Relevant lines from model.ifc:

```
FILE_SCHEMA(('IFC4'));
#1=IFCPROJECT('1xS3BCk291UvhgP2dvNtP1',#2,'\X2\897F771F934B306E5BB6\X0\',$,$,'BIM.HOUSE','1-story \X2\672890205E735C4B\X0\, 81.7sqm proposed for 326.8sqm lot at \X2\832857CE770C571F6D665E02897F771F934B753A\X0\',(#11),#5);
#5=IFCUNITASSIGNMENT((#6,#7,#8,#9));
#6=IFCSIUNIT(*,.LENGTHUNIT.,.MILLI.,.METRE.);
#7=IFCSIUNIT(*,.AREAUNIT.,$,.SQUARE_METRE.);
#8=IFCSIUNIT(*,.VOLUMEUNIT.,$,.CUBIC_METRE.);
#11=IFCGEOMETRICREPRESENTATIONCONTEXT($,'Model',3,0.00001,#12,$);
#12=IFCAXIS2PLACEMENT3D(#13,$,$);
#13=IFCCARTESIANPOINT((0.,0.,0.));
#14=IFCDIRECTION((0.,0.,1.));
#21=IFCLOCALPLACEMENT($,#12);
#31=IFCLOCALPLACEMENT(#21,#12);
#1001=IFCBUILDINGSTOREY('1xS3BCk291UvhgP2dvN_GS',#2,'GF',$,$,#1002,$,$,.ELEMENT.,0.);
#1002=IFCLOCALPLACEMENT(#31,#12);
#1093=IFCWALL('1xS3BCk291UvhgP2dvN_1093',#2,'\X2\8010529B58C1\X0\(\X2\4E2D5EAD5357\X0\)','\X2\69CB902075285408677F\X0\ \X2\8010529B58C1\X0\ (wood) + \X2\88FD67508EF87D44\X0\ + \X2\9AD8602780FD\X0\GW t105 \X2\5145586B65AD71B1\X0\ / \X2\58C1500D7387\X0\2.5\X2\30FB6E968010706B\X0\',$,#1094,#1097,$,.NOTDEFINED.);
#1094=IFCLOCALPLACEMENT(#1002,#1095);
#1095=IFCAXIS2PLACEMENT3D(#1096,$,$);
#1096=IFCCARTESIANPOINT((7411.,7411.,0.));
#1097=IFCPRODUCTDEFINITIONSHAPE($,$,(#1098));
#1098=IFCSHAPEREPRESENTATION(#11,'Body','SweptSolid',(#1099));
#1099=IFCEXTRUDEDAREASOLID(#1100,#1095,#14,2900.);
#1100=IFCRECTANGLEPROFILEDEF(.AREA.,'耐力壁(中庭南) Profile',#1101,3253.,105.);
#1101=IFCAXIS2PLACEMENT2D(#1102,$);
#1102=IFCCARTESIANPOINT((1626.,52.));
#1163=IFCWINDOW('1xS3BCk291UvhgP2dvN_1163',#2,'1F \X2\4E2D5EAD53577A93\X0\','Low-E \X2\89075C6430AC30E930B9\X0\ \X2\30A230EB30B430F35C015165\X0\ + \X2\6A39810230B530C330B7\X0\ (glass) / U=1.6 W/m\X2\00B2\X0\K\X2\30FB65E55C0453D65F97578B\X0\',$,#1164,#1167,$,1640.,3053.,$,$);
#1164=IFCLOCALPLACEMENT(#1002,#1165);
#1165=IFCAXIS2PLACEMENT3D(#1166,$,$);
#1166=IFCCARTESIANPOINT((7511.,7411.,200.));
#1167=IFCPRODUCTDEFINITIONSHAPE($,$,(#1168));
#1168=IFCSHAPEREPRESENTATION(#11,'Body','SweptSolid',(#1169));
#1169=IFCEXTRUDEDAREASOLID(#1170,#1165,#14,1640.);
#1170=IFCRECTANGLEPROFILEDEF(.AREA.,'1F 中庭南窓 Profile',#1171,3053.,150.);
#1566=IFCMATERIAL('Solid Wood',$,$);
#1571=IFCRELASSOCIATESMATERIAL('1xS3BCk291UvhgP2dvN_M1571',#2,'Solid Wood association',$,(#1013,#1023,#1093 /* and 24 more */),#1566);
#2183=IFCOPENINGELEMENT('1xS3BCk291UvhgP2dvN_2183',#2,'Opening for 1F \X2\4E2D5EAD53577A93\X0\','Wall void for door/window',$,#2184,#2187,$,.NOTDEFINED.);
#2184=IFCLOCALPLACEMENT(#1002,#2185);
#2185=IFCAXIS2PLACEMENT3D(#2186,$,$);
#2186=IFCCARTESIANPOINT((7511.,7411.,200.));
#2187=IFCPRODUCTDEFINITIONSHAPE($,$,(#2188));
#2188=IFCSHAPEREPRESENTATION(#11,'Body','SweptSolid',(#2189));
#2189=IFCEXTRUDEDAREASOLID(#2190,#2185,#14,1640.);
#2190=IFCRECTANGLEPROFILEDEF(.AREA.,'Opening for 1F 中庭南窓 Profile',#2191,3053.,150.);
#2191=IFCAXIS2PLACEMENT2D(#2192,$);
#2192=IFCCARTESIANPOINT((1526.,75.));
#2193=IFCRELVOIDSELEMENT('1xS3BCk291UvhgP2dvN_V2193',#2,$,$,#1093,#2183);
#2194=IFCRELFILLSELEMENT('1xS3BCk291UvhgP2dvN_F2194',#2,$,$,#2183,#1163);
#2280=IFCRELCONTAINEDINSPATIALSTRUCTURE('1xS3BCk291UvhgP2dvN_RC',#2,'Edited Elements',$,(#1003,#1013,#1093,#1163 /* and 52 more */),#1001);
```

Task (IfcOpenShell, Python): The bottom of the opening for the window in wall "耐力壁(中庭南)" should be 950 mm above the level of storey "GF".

```python
import numpy as np
import ifcopenshell
import ifcopenshell.api.geometry
import ifcopenshell.geom
import ifcopenshell.util.element
import ifcopenshell.util.placement
import ifcopenshell.util.shape
import ifcopenshell.util.unit

model = ifcopenshell.open("model.ifc")
unit_scale = ifcopenshell.util.unit.calculate_unit_scale(model)

window = model.by_id(1163)
opening = window.FillsVoids[0].RelatingOpeningElement
storey = ifcopenshell.util.element.get_container(window, ifc_class="IfcBuildingStorey")
level = ifcopenshell.util.placement.get_local_placement(storey.ObjectPlacement)[2, 3]

# The opening's origin need not be at the sill, so measure its lowest point.
shape = ifcopenshell.geom.create_shape(ifcopenshell.geom.settings(), opening)
bottom = ifcopenshell.util.shape.get_shape_bottom_elevation(shape, shape.geometry) / unit_scale
dz = level + 0.95 / unit_scale - bottom

shift = np.array([0.0, 0.0, dz])
# The window is not placed relative to its opening, so move both.
for product in (opening, window):
    matrix = ifcopenshell.util.placement.get_local_placement(product.ObjectPlacement)
    matrix[:3, 3] += shift
    ifcopenshell.api.geometry.edit_object_placement(model, product=product, matrix=matrix, is_si=False)

print(f"moved by {dz * unit_scale:+.3f} m")

model.write("model_v2.ifc")
```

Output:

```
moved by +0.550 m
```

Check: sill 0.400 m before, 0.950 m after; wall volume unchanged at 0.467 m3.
